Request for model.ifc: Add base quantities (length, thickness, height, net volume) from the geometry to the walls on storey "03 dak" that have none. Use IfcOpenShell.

First a look at what the model holds.

```python
import ifcopenshell
import ifcopenshell.util.element
import ifcopenshell.util.unit

model = ifcopenshell.open("model.ifc")
print(model.schema)
for unit_type in ("LENGTHUNIT", "AREAUNIT", "VOLUMEUNIT"):
    print(unit_type, ifcopenshell.util.unit.calculate_unit_scale(model, unit_type))
storey = next(s for s in model.by_type("IfcBuildingStorey") if s.Name == "03 dak")
walls = [e for e in ifcopenshell.util.element.get_decomposition(storey) if e.is_a("IfcWall")]
for e in sorted(walls, key=lambda e: e.id()):
    print(e.id(), e.is_a(), e.Name, list(ifcopenshell.util.element.get_psets(e, qtos_only=True)), sep=" | ")
```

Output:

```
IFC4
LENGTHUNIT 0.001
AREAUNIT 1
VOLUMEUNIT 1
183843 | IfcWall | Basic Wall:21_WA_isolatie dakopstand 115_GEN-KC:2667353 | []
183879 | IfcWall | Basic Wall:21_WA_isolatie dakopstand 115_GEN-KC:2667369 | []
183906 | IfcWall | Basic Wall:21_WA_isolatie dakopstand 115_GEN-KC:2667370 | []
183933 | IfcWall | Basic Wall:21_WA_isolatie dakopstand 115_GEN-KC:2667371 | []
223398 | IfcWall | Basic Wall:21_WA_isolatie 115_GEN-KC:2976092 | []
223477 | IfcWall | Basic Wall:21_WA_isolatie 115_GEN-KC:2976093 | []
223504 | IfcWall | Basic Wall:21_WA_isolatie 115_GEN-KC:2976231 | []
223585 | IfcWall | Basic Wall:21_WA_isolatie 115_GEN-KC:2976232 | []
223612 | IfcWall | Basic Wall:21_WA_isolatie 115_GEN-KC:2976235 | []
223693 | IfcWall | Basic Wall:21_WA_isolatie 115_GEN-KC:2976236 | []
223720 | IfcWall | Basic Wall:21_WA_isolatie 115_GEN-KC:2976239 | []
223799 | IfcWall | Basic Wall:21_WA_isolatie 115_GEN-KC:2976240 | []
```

```python
import ifcopenshell
import ifcopenshell.api.pset
import ifcopenshell.geom
import ifcopenshell.util.element
import ifcopenshell.util.shape
import ifcopenshell.util.unit

model = ifcopenshell.open("model.ifc")
unit_scale = ifcopenshell.util.unit.calculate_unit_scale(model)
volume_scale = ifcopenshell.util.unit.calculate_unit_scale(model, "VOLUMEUNIT")
settings = ifcopenshell.geom.settings()

storey = next(s for s in model.by_type("IfcBuildingStorey") if s.Name == "03 dak")
walls = [e for e in ifcopenshell.util.element.get_decomposition(storey) if e.is_a("IfcWall")]

for e in sorted(walls, key=lambda e: e.id()):
    if ifcopenshell.util.element.get_psets(e, qtos_only=True, should_inherit=False):
        continue
    # Geometry comes back in metres, in the element's own axes.
    shape = ifcopenshell.geom.create_shape(settings, e)
    values = {
        "Length": ifcopenshell.util.shape.get_x(shape.geometry) / unit_scale,
        "Width": ifcopenshell.util.shape.get_y(shape.geometry) / unit_scale,
        "Height": ifcopenshell.util.shape.get_z(shape.geometry) / unit_scale,
        "NetVolume": ifcopenshell.util.shape.get_volume(shape.geometry) / volume_scale,
    }
    qto = ifcopenshell.api.pset.add_qto(model, product=e, name="Qto_WallBaseQuantities")
    ifcopenshell.api.pset.edit_qto(model, qto=qto, properties=values)
    print(e.id(), {k: round(v, 3) for k, v in values.items()})

model.write("model_rev.ifc")
```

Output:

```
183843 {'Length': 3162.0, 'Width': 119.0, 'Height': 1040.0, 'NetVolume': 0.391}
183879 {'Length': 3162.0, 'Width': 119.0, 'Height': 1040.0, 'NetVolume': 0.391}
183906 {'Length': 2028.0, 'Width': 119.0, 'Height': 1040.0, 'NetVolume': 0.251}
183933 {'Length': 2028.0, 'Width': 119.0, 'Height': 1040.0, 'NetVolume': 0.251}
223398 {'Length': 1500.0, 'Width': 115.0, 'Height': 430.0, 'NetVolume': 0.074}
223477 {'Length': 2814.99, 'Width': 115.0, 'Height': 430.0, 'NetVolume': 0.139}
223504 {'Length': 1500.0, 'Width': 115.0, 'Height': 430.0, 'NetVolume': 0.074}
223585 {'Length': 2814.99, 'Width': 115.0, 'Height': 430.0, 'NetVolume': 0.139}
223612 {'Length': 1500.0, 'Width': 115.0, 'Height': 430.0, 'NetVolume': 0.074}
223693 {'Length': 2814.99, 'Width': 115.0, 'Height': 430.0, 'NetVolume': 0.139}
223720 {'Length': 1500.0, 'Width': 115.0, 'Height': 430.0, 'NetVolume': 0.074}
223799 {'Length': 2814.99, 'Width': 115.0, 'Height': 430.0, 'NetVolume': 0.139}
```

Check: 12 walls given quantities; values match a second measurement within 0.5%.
